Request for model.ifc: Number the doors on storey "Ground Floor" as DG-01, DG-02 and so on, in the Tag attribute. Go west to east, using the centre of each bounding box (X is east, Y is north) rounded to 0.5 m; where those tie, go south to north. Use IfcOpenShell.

First a look at what the model holds.

```python
import ifcopenshell
import ifcopenshell.util.element
import ifcopenshell.util.placement

model = ifcopenshell.open("model.ifc")
print(model.schema)
storey = next(s for s in model.by_type("IfcBuildingStorey") if s.Name == "Ground Floor")
doors = [e for e in ifcopenshell.util.element.get_decomposition(storey) if e.is_a("IfcDoor")]
for e in sorted(doors, key=lambda e: e.id()):
    origin = ifcopenshell.util.placement.get_local_placement(e.ObjectPlacement)[:3, 3]
    print(e.id(), e.Tag, e.Name, origin.round(2) + 0.0, sep=" | ")
```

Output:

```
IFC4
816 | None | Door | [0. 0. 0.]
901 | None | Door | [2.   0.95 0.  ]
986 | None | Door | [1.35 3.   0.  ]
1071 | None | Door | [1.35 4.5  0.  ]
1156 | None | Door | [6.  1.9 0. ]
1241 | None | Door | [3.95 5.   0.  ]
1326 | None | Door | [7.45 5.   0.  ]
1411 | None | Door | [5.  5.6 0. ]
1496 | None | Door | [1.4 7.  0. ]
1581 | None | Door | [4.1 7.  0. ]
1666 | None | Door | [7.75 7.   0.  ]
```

```python
import ifcopenshell
import ifcopenshell.geom
import ifcopenshell.util.element
import ifcopenshell.util.shape

model = ifcopenshell.open("model.ifc")
settings = ifcopenshell.geom.settings()
settings.set("use-world-coords", True)


def centre(element):
    shape = ifcopenshell.geom.create_shape(settings, element)
    return ifcopenshell.util.shape.get_bbox_centroid(shape.geometry)


storey = next(s for s in model.by_type("IfcBuildingStorey") if s.Name == "Ground Floor")
doors = [e for e in ifcopenshell.util.element.get_decomposition(storey) if e.is_a("IfcDoor")]

# Insertion points can sit at a corner or the storey origin, so sort by the geometry (in metres).
centres = {e: centre(e) for e in doors}
doors.sort(key=lambda e: (round(centres[e][0] / 0.5), centres[e][1]))

for i, e in enumerate(doors, start=1):
    number = f"DG-{i:02d}"
    e.Tag = number
    print(e.id(), number)

model.write("model-out.ifc")
```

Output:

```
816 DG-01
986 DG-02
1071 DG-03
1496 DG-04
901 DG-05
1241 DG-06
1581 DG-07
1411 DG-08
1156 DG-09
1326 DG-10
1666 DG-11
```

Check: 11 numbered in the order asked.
